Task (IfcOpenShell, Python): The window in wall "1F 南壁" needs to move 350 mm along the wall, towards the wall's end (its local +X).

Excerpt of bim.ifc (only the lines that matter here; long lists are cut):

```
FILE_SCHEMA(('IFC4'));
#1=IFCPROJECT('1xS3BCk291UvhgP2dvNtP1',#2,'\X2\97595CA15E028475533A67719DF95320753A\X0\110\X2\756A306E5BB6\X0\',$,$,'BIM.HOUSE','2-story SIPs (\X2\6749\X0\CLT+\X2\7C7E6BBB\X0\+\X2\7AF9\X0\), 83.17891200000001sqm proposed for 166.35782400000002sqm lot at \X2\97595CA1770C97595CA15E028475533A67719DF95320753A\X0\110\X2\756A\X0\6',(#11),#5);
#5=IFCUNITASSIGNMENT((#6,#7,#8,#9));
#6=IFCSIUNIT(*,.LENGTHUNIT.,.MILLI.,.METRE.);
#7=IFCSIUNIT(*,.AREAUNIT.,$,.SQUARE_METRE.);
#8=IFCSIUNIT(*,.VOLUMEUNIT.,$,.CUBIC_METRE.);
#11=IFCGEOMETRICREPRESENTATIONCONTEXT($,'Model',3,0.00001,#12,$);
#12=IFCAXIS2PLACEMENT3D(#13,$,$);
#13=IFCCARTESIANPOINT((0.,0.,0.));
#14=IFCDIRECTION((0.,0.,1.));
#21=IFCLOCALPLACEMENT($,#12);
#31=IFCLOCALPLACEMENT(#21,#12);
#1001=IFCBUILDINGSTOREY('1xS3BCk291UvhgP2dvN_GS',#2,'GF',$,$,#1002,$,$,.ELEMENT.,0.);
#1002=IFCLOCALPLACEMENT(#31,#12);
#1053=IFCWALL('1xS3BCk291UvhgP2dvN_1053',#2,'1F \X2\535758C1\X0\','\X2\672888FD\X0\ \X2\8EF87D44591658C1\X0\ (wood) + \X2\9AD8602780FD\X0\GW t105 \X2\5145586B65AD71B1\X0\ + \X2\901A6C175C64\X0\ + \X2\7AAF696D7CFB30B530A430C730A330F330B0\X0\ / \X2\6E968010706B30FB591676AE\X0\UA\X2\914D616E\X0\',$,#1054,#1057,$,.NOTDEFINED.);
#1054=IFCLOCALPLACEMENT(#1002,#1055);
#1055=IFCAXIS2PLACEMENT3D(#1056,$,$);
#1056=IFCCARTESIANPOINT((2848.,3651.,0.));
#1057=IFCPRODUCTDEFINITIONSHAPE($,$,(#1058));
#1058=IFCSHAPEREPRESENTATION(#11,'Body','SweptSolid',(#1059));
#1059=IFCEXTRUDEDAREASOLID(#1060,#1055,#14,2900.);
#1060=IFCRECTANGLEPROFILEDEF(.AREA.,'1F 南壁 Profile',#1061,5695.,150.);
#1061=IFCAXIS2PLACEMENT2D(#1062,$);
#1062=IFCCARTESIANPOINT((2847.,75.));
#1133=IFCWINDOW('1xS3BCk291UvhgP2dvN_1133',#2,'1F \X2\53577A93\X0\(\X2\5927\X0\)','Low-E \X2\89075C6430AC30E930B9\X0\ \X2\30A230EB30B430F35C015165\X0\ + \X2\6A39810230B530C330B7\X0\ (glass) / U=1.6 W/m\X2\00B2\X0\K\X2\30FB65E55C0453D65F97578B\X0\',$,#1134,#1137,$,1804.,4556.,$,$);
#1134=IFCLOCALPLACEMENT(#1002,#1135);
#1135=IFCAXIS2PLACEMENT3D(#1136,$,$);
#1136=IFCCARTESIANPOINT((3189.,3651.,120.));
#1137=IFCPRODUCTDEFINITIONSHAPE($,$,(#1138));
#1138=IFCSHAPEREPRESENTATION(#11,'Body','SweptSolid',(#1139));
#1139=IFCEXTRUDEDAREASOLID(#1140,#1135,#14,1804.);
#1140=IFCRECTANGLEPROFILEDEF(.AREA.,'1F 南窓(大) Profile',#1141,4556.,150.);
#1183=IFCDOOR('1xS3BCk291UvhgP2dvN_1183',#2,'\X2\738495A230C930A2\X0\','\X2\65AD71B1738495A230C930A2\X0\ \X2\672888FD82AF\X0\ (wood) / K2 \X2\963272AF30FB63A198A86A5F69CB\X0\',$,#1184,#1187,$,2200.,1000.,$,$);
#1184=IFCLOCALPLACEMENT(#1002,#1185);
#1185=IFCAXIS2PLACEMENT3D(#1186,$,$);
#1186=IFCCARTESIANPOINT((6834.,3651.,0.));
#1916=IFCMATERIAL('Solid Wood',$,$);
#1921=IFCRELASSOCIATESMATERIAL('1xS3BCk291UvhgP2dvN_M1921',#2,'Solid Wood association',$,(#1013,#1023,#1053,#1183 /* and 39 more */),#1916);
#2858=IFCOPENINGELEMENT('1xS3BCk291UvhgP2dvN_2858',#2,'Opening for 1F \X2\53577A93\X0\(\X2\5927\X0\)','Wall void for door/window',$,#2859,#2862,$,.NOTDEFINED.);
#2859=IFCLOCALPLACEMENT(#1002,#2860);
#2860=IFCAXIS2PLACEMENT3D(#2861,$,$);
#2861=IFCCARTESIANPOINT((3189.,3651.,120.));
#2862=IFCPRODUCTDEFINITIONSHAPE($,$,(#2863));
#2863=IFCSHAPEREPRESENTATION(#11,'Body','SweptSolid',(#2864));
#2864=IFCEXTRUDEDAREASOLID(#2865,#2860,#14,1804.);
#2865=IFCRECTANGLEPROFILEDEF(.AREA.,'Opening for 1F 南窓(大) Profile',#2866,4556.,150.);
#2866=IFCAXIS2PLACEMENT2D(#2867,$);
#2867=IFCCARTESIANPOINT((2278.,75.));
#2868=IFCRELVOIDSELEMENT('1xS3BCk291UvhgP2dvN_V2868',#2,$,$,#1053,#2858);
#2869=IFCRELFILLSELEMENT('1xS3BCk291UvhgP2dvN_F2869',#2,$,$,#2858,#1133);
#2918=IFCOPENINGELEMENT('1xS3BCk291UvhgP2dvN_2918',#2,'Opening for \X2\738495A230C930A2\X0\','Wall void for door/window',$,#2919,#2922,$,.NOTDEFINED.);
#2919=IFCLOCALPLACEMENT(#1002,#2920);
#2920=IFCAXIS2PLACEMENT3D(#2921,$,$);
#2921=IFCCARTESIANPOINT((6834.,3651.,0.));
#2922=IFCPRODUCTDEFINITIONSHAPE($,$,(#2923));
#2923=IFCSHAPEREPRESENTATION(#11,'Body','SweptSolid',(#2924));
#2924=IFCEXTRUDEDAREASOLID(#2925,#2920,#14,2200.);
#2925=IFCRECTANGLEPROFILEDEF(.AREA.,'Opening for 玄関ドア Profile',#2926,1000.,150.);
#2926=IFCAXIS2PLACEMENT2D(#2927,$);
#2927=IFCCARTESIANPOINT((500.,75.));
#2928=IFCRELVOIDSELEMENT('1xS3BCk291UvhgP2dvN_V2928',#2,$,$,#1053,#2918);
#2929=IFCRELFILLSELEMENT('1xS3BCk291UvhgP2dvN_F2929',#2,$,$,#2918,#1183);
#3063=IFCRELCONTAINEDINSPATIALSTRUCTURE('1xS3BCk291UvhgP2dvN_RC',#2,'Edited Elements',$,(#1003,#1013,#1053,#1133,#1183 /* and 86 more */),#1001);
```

```python
import ifcopenshell
import ifcopenshell.api.geometry
import ifcopenshell.util.placement

model = ifcopenshell.open("bim.ifc")

window = model.by_guid("1xS3BCk291UvhgP2dvN_1133")
opening = window.FillsVoids[0].RelatingOpeningElement
wall = opening.VoidsElements[0].RelatingBuildingElement

wall_matrix = ifcopenshell.util.placement.get_local_placement(wall.ObjectPlacement)
shift = wall_matrix[:3, 0] * 350.0
before = ifcopenshell.util.placement.get_local_placement(window.ObjectPlacement)[:3, 3].copy()

# The window is not placed relative to its opening, so move both.
for product in (opening, window):
    matrix = ifcopenshell.util.placement.get_local_placement(product.ObjectPlacement)
    matrix[:3, 3] += shift
    ifcopenshell.api.geometry.edit_object_placement(model, product=product, matrix=matrix, is_si=False)

after = ifcopenshell.util.placement.get_local_placement(window.ObjectPlacement)[:3, 3]
print("window moved by", (after - before).round(3) + 0.0)

model.write("bim_edited.ifc")
```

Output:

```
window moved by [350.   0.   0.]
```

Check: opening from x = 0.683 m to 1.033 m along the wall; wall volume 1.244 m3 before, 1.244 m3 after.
